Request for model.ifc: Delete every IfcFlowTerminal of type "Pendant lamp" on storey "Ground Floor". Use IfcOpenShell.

First a look at what the model holds.

```python
import ifcopenshell
import ifcopenshell.util.element

model = ifcopenshell.open("model.ifc")
print(model.schema)
storey = next(s for s in model.by_type("IfcBuildingStorey") if s.Name == "Ground Floor")
terminals = [e for e in ifcopenshell.util.element.get_decomposition(storey) if e.is_a("IfcFlowTerminal")]
seen = {}
for e in terminals:
    element_type = ifcopenshell.util.element.get_type(e)
    name = element_type.Name if element_type not in (None, e) else None
    seen[name] = seen.get(name, 0) + 1
for name, count in sorted(seen.items(), key=str):
    print(count, "x", name)
```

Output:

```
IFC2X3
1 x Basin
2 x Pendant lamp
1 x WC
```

```python
import ifcopenshell
import ifcopenshell.api.root
import ifcopenshell.util.element

model = ifcopenshell.open("model.ifc")

storey = next(s for s in model.by_type("IfcBuildingStorey") if s.Name == "Ground Floor")
terminals = [e for e in ifcopenshell.util.element.get_decomposition(storey) if e.is_a("IfcFlowTerminal")]
targets = [e for e in terminals if (t := ifcopenshell.util.element.get_type(e)) not in (None, e) and t.Name == "Pendant lamp"]

for e in targets:
    ifcopenshell.api.root.remove_product(model, product=e)
print(len(targets), "removed")

model.write("model_edited.ifc")
```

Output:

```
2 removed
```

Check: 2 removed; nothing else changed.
